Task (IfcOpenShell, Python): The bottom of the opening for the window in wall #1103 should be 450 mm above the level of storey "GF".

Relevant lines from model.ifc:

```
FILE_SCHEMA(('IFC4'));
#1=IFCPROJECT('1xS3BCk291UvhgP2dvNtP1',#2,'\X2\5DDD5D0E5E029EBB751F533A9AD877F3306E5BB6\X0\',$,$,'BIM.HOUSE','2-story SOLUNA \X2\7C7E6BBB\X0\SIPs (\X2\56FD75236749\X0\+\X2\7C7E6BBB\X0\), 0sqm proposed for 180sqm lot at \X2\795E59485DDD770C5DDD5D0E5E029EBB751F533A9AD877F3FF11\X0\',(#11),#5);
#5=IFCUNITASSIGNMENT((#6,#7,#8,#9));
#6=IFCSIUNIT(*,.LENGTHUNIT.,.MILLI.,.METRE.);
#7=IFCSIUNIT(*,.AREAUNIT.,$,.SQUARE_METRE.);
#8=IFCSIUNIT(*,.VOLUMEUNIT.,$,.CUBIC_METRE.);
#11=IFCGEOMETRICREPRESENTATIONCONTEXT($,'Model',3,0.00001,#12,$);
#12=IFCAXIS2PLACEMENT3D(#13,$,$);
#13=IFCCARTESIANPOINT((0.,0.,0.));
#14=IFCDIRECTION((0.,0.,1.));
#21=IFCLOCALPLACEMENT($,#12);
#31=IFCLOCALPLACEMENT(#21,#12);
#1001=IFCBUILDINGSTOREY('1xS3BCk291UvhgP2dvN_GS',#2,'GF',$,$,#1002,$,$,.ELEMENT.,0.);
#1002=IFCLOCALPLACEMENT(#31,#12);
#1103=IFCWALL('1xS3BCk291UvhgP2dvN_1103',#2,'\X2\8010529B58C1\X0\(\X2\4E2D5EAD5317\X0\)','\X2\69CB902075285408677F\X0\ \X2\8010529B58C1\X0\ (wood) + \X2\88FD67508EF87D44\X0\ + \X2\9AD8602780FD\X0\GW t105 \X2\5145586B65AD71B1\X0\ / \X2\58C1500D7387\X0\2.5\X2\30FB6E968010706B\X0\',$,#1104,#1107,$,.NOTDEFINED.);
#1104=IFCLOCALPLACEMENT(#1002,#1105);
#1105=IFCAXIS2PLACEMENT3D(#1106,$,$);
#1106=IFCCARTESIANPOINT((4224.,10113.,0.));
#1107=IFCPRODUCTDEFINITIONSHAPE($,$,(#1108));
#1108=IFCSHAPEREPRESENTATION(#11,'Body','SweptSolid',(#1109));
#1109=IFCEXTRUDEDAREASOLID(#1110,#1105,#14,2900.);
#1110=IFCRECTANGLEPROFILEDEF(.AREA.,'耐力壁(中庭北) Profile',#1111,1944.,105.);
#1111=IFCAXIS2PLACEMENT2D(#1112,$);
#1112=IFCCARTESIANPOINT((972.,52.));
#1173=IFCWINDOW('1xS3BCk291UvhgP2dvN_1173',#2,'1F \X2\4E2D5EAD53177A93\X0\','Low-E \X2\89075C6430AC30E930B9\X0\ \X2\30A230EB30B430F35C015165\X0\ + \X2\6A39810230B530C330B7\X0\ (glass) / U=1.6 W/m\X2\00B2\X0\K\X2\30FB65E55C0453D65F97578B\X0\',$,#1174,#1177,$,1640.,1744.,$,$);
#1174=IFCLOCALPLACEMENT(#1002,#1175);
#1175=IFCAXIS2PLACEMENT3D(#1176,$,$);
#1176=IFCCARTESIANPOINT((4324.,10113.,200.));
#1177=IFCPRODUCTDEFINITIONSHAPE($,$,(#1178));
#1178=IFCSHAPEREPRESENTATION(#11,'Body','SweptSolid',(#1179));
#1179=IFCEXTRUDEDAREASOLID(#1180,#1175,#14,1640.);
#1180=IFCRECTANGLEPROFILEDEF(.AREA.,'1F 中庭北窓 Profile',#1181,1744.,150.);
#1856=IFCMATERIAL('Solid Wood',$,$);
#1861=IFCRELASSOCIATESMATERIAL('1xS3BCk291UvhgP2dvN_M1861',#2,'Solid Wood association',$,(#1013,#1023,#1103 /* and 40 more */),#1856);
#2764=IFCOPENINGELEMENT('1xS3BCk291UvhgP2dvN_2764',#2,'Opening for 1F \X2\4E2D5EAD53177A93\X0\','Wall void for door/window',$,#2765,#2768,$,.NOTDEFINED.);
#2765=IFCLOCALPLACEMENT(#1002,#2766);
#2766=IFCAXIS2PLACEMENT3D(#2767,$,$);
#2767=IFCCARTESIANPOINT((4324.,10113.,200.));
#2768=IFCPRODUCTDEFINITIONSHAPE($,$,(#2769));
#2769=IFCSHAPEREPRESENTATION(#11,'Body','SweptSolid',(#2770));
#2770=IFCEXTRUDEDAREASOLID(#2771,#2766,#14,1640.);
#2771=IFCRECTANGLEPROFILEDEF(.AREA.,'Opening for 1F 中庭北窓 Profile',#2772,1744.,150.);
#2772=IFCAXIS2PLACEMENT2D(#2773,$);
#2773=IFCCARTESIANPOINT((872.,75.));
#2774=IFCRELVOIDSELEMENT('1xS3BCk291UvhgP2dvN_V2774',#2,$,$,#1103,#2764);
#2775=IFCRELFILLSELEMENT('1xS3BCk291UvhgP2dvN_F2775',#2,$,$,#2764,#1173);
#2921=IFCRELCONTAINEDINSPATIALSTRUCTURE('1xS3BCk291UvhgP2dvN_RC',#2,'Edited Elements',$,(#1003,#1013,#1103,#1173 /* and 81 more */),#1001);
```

```python
import numpy as np
import ifcopenshell
import ifcopenshell.api.geometry
import ifcopenshell.geom
import ifcopenshell.util.element
import ifcopenshell.util.placement
import ifcopenshell.util.shape
import ifcopenshell.util.unit

model = ifcopenshell.open("model.ifc")
unit_scale = ifcopenshell.util.unit.calculate_unit_scale(model)

window = model.by_id(1173)
opening = window.FillsVoids[0].RelatingOpeningElement
storey = ifcopenshell.util.element.get_container(window, ifc_class="IfcBuildingStorey")
level = ifcopenshell.util.placement.get_local_placement(storey.ObjectPlacement)[2, 3]

# The opening's origin need not be at the sill, so measure its lowest point.
shape = ifcopenshell.geom.create_shape(ifcopenshell.geom.settings(), opening)
bottom = ifcopenshell.util.shape.get_shape_bottom_elevation(shape, shape.geometry) / unit_scale
dz = level + 450.0 - bottom

shift = np.array([0.0, 0.0, dz])
# The window is not placed relative to its opening, so move both.
for product in (opening, window):
    matrix = ifcopenshell.util.placement.get_local_placement(product.ObjectPlacement)
    matrix[:3, 3] += shift
    ifcopenshell.api.geometry.edit_object_placement(model, product=product, matrix=matrix, is_si=False)

print(f"moved by {dz * unit_scale:+.3f} m")

model.write("model_v2.ifc")
```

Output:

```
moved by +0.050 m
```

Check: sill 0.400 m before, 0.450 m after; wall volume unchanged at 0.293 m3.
